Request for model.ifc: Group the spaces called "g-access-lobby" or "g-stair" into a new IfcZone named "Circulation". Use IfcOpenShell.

First a look at what the model holds.

```python
import ifcopenshell

model = ifcopenshell.open("model.ifc")
print(model.schema)
seen = {}
for space in model.by_type("IfcSpace"):
    seen[space.LongName] = seen.get(space.LongName, 0) + 1
for name, count in sorted(seen.items(), key=str):
    print(count, "x", name)
print("zones:", [z.Name for z in model.by_type("IfcZone")][:20])
```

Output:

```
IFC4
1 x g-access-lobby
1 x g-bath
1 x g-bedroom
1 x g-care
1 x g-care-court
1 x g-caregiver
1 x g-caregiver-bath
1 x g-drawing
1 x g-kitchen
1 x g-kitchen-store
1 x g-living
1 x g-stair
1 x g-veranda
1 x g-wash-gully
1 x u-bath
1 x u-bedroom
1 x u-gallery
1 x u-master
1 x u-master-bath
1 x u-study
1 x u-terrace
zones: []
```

```python
import ifcopenshell
import ifcopenshell.api.group
import ifcopenshell.api.root

model = ifcopenshell.open("model.ifc")

names = {"g-access-lobby", "g-stair"}
spaces = [s for s in model.by_type("IfcSpace") if s.LongName in names]

zone = ifcopenshell.api.root.create_entity(model, ifc_class="IfcZone", name="Circulation")
ifcopenshell.api.group.assign_group(model, products=spaces, group=zone)
print(len(spaces), "spaces in", zone.Name)

model.write("model-out.ifc")
```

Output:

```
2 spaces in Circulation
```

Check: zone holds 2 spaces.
